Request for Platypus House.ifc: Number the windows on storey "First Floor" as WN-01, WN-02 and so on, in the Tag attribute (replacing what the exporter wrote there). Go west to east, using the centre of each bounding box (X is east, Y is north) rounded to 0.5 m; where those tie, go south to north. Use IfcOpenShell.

First a look at what the model holds.

```python
import ifcopenshell
import ifcopenshell.util.element
import ifcopenshell.util.placement

model = ifcopenshell.open("Platypus House.ifc")
print(model.schema)
storey = next(s for s in model.by_type("IfcBuildingStorey") if s.Name == "First Floor")
windows = [e for e in ifcopenshell.util.element.get_decomposition(storey) if e.is_a("IfcWindow")]
for e in sorted(windows, key=lambda e: e.id()):
    origin = ifcopenshell.util.placement.get_local_placement(e.ObjectPlacement)[:3, 3]
    print(e.id(), e.Tag, e.Name, origin.round(2) + 0.0, sep=" | ")
```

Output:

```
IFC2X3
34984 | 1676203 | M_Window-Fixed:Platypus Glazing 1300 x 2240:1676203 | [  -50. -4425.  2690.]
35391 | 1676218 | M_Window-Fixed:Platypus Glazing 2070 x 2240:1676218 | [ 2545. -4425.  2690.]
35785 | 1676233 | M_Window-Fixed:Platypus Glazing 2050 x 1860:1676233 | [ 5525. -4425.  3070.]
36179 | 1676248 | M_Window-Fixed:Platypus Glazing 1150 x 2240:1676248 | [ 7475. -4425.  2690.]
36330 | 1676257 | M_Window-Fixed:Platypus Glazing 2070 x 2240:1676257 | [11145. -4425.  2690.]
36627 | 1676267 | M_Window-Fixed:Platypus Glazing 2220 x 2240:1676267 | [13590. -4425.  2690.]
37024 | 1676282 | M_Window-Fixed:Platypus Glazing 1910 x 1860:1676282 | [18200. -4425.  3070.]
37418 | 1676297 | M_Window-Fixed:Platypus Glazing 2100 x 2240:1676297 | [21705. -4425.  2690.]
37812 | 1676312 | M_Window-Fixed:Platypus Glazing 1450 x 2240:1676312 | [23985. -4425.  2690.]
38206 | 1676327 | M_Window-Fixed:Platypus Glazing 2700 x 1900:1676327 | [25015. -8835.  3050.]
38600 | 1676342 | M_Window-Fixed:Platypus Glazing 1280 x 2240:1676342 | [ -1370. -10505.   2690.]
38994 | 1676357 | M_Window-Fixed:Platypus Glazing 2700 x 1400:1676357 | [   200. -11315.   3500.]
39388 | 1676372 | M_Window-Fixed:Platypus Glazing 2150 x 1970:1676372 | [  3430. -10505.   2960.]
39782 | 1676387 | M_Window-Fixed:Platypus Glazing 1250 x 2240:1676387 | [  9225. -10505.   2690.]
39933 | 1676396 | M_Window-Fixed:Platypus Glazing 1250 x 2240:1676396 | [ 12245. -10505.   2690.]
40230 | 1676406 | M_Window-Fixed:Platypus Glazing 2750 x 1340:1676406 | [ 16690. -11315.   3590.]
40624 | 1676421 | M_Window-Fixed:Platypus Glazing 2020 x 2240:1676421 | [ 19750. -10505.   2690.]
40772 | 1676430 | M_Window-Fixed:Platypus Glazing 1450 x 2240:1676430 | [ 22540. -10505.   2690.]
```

```python
import ifcopenshell
import ifcopenshell.geom
import ifcopenshell.util.element
import ifcopenshell.util.shape

model = ifcopenshell.open("Platypus House.ifc")
settings = ifcopenshell.geom.settings()
settings.set("use-world-coords", True)


def centre(element):
    shape = ifcopenshell.geom.create_shape(settings, element)
    return ifcopenshell.util.shape.get_bbox_centroid(shape.geometry)


storey = next(s for s in model.by_type("IfcBuildingStorey") if s.Name == "First Floor")
windows = [e for e in ifcopenshell.util.element.get_decomposition(storey) if e.is_a("IfcWindow")]

# Insertion points can sit at a corner or the storey origin, so sort by the geometry (in metres).
centres = {e: centre(e) for e in windows}
windows.sort(key=lambda e: (round(centres[e][0] / 0.5), centres[e][1]))

for i, e in enumerate(windows, start=1):
    number = f"WN-{i:02d}"
    e.Tag = number
    print(e.id(), number)

model.write("Platypus House-out.ifc")
```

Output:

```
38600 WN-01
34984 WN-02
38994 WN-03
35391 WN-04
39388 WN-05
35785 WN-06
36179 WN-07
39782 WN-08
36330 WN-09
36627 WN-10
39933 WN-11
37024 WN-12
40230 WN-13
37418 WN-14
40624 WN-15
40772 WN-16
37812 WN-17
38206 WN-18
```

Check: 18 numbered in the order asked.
